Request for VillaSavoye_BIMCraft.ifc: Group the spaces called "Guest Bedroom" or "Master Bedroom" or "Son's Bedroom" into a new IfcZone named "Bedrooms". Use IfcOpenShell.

First a look at what the model holds.

```python
import ifcopenshell

model = ifcopenshell.open("VillaSavoye_BIMCraft.ifc")
print(model.schema)
seen = {}
for space in model.by_type("IfcSpace"):
    seen[space.LongName] = seen.get(space.LongName, 0) + 1
for name, count in sorted(seen.items(), key=str):
    print(count, "x", name)
print("zones:", [z.Name for z in model.by_type("IfcZone")][:20])
```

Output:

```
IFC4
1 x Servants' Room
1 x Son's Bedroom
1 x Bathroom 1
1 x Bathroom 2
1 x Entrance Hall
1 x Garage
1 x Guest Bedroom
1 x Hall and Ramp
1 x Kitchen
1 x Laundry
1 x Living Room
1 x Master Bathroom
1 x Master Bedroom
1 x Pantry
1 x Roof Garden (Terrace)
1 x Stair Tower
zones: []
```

```python
import ifcopenshell
import ifcopenshell.api.group
import ifcopenshell.api.root

model = ifcopenshell.open("VillaSavoye_BIMCraft.ifc")

names = {"Guest Bedroom", "Master Bedroom", "Son's Bedroom"}
spaces = [s for s in model.by_type("IfcSpace") if s.LongName in names]

zone = ifcopenshell.api.root.create_entity(model, ifc_class="IfcZone", name="Bedrooms")
ifcopenshell.api.group.assign_group(model, products=spaces, group=zone)
print(len(spaces), "spaces in", zone.Name)

model.write("VillaSavoye_BIMCraft-out.ifc")
```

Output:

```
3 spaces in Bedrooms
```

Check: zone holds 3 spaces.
